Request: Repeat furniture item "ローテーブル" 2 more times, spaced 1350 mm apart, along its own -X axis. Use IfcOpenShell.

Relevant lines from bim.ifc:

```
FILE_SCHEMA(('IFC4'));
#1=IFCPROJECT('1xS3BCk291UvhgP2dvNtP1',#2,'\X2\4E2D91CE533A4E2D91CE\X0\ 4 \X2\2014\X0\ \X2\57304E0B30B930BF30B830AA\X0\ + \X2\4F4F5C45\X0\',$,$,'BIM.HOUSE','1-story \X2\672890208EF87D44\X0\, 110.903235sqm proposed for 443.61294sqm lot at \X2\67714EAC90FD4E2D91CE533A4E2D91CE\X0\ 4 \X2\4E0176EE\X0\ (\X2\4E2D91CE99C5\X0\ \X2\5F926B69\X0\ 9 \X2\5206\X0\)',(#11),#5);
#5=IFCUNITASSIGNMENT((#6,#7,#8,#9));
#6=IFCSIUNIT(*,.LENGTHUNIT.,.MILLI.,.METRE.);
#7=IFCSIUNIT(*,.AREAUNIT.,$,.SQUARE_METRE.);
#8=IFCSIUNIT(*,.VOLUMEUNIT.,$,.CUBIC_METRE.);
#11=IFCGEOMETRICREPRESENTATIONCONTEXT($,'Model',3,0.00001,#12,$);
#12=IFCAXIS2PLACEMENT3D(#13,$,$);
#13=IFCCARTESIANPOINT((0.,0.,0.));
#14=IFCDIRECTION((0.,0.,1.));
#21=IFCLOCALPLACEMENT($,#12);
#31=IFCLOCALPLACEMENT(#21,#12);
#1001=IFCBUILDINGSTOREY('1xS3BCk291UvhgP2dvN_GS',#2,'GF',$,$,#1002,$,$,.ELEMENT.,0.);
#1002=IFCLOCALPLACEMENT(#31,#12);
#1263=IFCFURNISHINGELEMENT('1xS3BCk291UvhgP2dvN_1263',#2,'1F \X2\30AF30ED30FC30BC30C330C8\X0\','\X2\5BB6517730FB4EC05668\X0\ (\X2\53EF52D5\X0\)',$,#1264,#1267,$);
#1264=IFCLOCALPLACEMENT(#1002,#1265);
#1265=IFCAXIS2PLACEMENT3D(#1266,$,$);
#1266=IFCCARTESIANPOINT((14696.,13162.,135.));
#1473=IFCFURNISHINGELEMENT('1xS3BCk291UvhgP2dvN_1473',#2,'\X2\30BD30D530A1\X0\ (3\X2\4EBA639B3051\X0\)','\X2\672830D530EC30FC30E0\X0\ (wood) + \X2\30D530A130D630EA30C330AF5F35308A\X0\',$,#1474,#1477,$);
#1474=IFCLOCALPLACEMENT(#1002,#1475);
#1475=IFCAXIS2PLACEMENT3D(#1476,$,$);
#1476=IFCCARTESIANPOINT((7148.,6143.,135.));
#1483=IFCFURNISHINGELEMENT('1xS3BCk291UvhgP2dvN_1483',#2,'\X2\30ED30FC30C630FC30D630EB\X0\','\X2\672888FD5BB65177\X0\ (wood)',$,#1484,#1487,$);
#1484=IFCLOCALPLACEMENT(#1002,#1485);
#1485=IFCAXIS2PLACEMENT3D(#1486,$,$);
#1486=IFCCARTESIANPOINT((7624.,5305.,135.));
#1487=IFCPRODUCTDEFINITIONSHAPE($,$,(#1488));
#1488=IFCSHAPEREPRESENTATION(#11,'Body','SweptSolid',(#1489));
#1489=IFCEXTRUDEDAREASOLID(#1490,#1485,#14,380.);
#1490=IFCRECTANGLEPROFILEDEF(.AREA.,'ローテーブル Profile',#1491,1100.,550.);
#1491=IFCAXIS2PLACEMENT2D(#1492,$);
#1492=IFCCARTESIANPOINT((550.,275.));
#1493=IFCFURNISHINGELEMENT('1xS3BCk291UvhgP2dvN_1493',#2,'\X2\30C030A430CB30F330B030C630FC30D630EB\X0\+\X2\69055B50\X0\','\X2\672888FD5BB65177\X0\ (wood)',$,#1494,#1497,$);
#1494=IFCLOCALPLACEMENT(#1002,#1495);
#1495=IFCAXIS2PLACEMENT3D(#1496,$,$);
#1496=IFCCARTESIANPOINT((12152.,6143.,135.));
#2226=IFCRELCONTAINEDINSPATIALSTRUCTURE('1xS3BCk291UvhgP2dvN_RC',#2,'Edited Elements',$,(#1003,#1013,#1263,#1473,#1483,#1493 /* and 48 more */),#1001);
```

```python
import ifcopenshell
import ifcopenshell.api.geometry
import ifcopenshell.api.root
import ifcopenshell.util.element
import ifcopenshell.util.placement

model = ifcopenshell.open("bim.ifc")


def reuse_history(source, copy):
    """copy_class also copies each property set's owner history, people and application; keep the originals."""
    for rel in copy.IsDefinedBy:
        if rel.is_a("IfcRelDefinesByProperties") and (history := rel.RelatingPropertyDefinition.OwnerHistory):
            rel.RelatingPropertyDefinition.OwnerHistory = source.OwnerHistory
            ifcopenshell.util.element.remove_deep2(model, history)


source = model.by_id(1483)
base = ifcopenshell.util.placement.get_local_placement(source.ObjectPlacement)
step = -base[:3, 0] * 1350.0

for i in range(1, 3):
    copy = ifcopenshell.api.root.copy_class(model, product=source)
    copy.Representation = ifcopenshell.util.element.copy_deep(
        model, source.Representation, exclude=["IfcGeometricRepresentationContext", "IfcRepresentationMap"]
    )
    reuse_history(source, copy)
    matrix = base.copy()
    matrix[:3, 3] += i * step
    print("added at", matrix[:3, 3].round(3) + 0.0)
    ifcopenshell.api.geometry.edit_object_placement(model, product=copy, matrix=matrix, is_si=False)

model.write("bim_updated.ifc")
```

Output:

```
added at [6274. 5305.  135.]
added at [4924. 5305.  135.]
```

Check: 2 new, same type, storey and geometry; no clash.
